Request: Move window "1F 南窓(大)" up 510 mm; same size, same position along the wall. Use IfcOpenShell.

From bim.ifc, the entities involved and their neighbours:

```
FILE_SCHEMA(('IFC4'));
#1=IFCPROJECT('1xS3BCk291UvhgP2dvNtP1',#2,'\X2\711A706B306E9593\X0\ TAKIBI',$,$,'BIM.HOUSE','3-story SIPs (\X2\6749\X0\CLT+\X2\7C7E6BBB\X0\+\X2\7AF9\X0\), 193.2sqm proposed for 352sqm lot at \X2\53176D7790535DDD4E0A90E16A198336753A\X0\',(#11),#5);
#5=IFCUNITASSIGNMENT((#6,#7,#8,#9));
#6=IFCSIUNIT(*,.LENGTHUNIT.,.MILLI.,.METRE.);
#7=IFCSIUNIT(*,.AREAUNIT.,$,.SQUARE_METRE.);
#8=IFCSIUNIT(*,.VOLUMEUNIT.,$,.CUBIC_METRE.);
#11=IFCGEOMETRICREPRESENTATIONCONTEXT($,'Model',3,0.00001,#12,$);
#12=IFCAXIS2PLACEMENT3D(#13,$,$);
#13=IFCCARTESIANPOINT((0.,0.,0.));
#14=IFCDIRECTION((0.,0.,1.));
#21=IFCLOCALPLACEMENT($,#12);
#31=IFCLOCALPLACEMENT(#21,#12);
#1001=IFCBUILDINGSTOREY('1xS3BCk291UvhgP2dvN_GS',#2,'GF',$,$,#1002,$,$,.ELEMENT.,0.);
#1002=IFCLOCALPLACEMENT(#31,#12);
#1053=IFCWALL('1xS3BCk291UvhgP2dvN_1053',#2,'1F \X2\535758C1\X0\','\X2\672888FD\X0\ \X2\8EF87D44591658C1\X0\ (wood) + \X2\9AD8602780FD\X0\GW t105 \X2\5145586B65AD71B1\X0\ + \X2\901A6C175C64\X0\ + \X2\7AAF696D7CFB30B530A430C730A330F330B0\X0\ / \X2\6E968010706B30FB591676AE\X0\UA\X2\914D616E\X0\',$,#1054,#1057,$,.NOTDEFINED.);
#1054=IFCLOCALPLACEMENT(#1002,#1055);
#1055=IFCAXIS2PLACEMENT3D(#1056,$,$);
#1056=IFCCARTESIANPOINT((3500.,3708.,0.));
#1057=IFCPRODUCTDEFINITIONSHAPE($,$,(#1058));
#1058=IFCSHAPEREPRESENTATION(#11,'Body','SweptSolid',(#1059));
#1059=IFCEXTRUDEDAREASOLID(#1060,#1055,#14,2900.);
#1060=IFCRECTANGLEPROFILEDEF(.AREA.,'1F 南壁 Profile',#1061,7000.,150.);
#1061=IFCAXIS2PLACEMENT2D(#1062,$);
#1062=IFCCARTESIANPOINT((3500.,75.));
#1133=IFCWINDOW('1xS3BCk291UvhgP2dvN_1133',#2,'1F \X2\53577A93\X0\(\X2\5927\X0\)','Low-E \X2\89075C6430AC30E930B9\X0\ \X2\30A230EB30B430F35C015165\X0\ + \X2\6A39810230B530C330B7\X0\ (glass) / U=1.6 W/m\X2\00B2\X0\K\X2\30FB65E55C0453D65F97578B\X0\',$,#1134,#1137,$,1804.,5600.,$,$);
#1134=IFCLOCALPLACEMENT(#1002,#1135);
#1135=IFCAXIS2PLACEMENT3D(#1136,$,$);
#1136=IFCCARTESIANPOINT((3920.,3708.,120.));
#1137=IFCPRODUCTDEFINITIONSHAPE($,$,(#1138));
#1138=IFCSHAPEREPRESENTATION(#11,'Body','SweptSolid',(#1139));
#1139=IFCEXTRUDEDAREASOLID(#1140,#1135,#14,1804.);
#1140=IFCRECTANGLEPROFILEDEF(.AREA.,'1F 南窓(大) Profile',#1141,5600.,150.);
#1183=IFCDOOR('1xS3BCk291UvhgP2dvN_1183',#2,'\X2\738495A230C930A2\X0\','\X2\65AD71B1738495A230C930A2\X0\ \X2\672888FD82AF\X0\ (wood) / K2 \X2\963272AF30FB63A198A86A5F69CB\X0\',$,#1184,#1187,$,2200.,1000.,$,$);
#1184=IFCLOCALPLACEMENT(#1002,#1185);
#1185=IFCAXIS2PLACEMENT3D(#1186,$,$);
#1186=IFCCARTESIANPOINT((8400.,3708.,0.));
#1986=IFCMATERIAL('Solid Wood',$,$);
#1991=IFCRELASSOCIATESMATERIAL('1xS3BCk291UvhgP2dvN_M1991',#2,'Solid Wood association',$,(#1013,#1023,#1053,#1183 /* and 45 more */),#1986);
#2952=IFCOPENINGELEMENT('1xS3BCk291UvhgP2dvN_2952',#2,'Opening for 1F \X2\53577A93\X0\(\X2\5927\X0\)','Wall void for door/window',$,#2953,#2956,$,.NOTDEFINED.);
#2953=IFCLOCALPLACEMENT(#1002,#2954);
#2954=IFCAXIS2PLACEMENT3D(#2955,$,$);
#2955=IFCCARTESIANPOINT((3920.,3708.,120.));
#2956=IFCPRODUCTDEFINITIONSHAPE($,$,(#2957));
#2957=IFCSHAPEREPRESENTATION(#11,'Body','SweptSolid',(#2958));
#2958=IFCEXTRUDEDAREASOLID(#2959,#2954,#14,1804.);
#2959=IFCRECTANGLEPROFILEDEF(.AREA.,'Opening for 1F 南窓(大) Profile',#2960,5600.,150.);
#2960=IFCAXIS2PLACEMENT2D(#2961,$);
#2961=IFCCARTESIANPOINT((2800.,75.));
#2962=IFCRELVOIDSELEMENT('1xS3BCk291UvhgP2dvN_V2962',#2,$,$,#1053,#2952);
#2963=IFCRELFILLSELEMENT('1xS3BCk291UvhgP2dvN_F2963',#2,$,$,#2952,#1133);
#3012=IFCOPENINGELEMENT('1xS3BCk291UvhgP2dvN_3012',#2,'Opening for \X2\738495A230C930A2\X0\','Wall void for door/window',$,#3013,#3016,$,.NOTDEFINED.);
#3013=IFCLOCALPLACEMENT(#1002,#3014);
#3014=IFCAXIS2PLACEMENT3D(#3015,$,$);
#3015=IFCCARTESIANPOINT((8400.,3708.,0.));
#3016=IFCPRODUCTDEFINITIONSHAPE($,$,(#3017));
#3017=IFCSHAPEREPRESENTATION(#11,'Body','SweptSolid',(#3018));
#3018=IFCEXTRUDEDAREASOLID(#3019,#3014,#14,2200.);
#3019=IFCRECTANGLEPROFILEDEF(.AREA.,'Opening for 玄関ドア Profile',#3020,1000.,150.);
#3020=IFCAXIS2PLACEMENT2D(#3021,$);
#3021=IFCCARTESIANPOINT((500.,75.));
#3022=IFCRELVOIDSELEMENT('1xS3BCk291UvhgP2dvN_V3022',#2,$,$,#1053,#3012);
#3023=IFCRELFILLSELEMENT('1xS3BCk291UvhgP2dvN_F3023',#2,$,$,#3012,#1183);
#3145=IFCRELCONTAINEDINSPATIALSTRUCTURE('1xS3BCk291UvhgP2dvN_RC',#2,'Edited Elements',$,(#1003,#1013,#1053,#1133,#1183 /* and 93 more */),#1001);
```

```python
import numpy as np
import ifcopenshell
import ifcopenshell.api.geometry
import ifcopenshell.util.placement
import ifcopenshell.util.unit

model = ifcopenshell.open("bim.ifc")
unit_scale = ifcopenshell.util.unit.calculate_unit_scale(model)

window = model.by_guid("1xS3BCk291UvhgP2dvN_1133")
opening = window.FillsVoids[0].RelatingOpeningElement
dz = 510.0

shift = np.array([0.0, 0.0, dz])
# The window is not placed relative to its opening, so move both.
for product in (opening, window):
    matrix = ifcopenshell.util.placement.get_local_placement(product.ObjectPlacement)
    matrix[:3, 3] += shift
    ifcopenshell.api.geometry.edit_object_placement(model, product=product, matrix=matrix, is_si=False)

print(f"moved by {dz * unit_scale:+.3f} m")

model.write("bim_updated.ifc")
```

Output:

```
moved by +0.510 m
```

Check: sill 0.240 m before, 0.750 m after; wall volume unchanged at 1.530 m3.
